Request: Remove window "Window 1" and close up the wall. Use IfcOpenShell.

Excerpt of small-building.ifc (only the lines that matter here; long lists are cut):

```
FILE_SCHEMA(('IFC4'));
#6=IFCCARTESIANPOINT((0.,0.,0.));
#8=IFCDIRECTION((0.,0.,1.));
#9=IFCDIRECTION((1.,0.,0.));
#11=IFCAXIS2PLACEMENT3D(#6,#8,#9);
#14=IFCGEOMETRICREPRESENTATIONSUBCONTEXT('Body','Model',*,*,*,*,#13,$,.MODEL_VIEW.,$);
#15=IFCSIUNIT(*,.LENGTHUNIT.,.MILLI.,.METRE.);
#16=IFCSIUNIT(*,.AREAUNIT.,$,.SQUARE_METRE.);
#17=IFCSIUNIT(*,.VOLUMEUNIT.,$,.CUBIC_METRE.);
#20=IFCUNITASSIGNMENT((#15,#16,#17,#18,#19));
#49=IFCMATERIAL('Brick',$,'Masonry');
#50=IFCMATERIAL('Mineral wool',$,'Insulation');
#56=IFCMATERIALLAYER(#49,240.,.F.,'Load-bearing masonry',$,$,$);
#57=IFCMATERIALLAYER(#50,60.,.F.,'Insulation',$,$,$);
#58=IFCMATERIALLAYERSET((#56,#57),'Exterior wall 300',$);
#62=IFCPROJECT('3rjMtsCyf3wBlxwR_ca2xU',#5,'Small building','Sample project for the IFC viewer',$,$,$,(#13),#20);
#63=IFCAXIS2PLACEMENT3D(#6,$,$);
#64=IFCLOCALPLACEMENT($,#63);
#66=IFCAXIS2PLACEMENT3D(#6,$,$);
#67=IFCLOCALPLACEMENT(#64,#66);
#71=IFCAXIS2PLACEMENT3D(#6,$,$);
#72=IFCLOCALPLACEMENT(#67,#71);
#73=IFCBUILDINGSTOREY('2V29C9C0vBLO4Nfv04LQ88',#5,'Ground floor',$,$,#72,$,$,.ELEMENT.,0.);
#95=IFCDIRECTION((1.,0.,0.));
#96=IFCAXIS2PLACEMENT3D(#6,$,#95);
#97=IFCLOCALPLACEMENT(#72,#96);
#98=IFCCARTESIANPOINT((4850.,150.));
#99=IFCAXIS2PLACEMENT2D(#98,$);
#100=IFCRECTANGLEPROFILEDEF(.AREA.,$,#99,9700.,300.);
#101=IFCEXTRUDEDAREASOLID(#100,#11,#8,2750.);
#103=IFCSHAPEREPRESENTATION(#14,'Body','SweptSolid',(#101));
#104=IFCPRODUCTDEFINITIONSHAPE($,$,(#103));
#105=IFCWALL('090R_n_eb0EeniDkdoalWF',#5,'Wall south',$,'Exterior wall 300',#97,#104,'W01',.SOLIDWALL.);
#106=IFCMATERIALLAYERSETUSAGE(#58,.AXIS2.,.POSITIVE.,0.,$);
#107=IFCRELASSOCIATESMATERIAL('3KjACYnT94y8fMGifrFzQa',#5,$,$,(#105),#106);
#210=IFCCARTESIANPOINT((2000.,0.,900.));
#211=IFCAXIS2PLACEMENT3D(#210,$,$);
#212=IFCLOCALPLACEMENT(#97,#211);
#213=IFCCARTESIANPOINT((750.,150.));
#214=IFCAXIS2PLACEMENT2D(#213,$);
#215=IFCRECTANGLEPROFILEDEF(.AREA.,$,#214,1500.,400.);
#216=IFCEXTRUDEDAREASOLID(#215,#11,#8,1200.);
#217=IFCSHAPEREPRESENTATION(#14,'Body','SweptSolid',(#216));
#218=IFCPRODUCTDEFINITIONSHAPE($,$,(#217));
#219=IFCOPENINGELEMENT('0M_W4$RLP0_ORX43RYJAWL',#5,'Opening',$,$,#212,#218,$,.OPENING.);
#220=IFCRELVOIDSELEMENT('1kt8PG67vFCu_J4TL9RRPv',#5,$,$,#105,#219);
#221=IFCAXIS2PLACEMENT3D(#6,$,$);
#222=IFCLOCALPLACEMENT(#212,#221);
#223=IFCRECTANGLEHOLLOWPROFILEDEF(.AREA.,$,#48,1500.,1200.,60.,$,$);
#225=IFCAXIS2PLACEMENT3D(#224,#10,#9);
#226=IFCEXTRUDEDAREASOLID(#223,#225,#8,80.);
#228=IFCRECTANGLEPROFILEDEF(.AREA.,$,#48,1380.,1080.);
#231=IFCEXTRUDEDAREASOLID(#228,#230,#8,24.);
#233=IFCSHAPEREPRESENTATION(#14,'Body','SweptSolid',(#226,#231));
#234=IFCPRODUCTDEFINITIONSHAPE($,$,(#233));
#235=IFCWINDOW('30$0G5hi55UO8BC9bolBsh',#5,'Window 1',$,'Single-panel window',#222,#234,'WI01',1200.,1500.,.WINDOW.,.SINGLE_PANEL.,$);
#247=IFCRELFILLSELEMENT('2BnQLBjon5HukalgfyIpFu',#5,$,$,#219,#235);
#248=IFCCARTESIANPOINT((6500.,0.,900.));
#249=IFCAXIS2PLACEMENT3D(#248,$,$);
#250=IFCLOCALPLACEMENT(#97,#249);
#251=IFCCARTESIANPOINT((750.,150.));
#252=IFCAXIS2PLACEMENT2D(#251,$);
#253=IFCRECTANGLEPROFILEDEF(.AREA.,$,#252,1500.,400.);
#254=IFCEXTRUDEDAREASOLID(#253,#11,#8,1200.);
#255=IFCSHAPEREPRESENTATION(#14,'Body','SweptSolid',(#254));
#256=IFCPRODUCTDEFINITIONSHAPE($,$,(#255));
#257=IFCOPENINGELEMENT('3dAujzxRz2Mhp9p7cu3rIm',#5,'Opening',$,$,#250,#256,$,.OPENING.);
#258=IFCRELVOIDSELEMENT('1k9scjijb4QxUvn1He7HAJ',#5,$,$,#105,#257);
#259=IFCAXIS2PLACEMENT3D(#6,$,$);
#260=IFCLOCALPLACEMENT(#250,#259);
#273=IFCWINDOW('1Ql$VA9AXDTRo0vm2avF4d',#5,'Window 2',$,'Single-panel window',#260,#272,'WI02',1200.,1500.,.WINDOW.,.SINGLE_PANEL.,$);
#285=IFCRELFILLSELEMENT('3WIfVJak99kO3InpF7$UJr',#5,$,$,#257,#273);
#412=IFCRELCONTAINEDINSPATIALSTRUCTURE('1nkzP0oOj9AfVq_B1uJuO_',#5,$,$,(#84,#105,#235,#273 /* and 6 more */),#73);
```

```python
import ifcopenshell
import ifcopenshell.api.feature
import ifcopenshell.api.root
import ifcopenshell.geom
import ifcopenshell.util.shape

model = ifcopenshell.open("small-building.ifc")
settings = ifcopenshell.geom.settings()


def volume(element):
    """Net volume in cubic metres, openings subtracted."""
    shape = ifcopenshell.geom.create_shape(settings, element)
    return ifcopenshell.util.shape.get_volume(shape.geometry)


window = model.by_guid("30$0G5hi55UO8BC9bolBsh")
opening = window.FillsVoids[0].RelatingOpeningElement
wall = opening.VoidsElements[0].RelatingBuildingElement
before = volume(wall)

ifcopenshell.api.root.remove_product(model, product=window)
ifcopenshell.api.feature.remove_feature(model, feature=opening)

after = volume(wall)

print(f"wall volume {before:.3f} -> {after:.3f} m3")

model.write("small-building_updated.ifc")
```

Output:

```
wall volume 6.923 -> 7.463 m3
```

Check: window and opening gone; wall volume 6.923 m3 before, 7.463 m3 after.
